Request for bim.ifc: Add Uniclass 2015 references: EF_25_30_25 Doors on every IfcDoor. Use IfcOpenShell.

First a look at what the model holds.

```python
import ifcopenshell

model = ifcopenshell.open("bim.ifc")
print(model.schema)
print("classifications:", [c.Name for c in model.by_type("IfcClassification")])
for ifc_class in ("IfcDoor", "IfcRoof", "IfcStair", "IfcWall", "IfcWindow"):
    print(ifc_class, len(model.by_type(ifc_class)))
```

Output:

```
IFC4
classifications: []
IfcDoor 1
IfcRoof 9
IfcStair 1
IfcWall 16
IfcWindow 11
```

```python
import ifcopenshell
import ifcopenshell.api.classification

model = ifcopenshell.open("bim.ifc")

system = ifcopenshell.api.classification.add_classification(model, classification="Uniclass 2015")

codes = {
    "IfcDoor": ("EF_25_30_25", "Doors"),
}
for ifc_class, (code, name) in codes.items():
    products = model.by_type(ifc_class)
    ifcopenshell.api.classification.add_reference(
        model, products=products, classification=system, identification=code, name=name
    )
    print(code, len(products))

model.write("bim_edited.ifc")
```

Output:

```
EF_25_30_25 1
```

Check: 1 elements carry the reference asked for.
